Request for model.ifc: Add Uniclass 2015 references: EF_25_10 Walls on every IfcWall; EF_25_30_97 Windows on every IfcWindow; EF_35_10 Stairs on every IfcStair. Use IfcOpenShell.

First a look at what the model holds.

```python
import ifcopenshell

model = ifcopenshell.open("model.ifc")
print(model.schema)
print("classifications:", [c.Name for c in model.by_type("IfcClassification")])
for ifc_class in ("IfcDoor", "IfcRoof", "IfcStair", "IfcWall", "IfcWindow"):
    print(ifc_class, len(model.by_type(ifc_class)))
```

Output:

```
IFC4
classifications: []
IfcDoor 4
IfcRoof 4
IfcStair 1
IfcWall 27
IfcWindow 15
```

```python
import ifcopenshell
import ifcopenshell.api.classification

model = ifcopenshell.open("model.ifc")

system = ifcopenshell.api.classification.add_classification(model, classification="Uniclass 2015")

codes = {
    "IfcWall": ("EF_25_10", "Walls"),
    "IfcWindow": ("EF_25_30_97", "Windows"),
    "IfcStair": ("EF_35_10", "Stairs"),
}
for ifc_class, (code, name) in codes.items():
    products = model.by_type(ifc_class)
    ifcopenshell.api.classification.add_reference(
        model, products=products, classification=system, identification=code, name=name
    )
    print(code, len(products))

model.write("model_updated.ifc")
```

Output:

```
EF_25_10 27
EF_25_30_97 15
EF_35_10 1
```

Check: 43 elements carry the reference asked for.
